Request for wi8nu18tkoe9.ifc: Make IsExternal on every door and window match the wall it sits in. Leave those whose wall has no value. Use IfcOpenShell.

First a look at what the model holds.

```python
import ifcopenshell
import ifcopenshell.util.element

model = ifcopenshell.open("wi8nu18tkoe9.ifc")
print(model.schema)
seen = {}
for e in model.by_type("IfcDoor") + model.by_type("IfcWindow"):
    if not e.FillsVoids:
        continue
    host = e.FillsVoids[0].RelatingOpeningElement.VoidsElements[0].RelatingBuildingElement
    own = ifcopenshell.util.element.get_pset(e, f"Pset_{e.is_a()[3:].removesuffix('StandardCase')}Common", "IsExternal")
    wall = ifcopenshell.util.element.get_pset(host, "Pset_WallCommon", "IsExternal")
    seen[e.is_a(), own, wall] = seen.get((e.is_a(), own, wall), 0) + 1
for (cls, own, wall), count in sorted(seen.items(), key=str):
    print(count, cls, "IsExternal:", own, "| host wall:", wall)
```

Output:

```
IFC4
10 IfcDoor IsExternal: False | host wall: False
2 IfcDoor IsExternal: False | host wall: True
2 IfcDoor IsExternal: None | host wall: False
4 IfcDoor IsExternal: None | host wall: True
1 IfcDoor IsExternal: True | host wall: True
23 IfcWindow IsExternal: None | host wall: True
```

```python
import ifcopenshell
import ifcopenshell.api.pset
import ifcopenshell.util.element

model = ifcopenshell.open("wi8nu18tkoe9.ifc")

count = 0
for ifc_class, pset_name in (("IfcDoor", "Pset_DoorCommon"), ("IfcWindow", "Pset_WindowCommon")):
    for e in model.by_type(ifc_class):
        if not e.FillsVoids:
            continue
        host = e.FillsVoids[0].RelatingOpeningElement.VoidsElements[0].RelatingBuildingElement
        external = ifcopenshell.util.element.get_pset(host, "Pset_WallCommon", "IsExternal")
        if external is None or ifcopenshell.util.element.get_pset(e, pset_name, "IsExternal") == external:
            continue
        pset = ifcopenshell.api.pset.add_pset(model, product=e, name=pset_name)
        ifcopenshell.api.pset.edit_pset(model, pset=pset, properties={"IsExternal": external})
        count += 1

print(count, "updated")

model.write("wi8nu18tkoe9_edited.ifc")
```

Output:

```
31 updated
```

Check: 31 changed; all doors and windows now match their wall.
